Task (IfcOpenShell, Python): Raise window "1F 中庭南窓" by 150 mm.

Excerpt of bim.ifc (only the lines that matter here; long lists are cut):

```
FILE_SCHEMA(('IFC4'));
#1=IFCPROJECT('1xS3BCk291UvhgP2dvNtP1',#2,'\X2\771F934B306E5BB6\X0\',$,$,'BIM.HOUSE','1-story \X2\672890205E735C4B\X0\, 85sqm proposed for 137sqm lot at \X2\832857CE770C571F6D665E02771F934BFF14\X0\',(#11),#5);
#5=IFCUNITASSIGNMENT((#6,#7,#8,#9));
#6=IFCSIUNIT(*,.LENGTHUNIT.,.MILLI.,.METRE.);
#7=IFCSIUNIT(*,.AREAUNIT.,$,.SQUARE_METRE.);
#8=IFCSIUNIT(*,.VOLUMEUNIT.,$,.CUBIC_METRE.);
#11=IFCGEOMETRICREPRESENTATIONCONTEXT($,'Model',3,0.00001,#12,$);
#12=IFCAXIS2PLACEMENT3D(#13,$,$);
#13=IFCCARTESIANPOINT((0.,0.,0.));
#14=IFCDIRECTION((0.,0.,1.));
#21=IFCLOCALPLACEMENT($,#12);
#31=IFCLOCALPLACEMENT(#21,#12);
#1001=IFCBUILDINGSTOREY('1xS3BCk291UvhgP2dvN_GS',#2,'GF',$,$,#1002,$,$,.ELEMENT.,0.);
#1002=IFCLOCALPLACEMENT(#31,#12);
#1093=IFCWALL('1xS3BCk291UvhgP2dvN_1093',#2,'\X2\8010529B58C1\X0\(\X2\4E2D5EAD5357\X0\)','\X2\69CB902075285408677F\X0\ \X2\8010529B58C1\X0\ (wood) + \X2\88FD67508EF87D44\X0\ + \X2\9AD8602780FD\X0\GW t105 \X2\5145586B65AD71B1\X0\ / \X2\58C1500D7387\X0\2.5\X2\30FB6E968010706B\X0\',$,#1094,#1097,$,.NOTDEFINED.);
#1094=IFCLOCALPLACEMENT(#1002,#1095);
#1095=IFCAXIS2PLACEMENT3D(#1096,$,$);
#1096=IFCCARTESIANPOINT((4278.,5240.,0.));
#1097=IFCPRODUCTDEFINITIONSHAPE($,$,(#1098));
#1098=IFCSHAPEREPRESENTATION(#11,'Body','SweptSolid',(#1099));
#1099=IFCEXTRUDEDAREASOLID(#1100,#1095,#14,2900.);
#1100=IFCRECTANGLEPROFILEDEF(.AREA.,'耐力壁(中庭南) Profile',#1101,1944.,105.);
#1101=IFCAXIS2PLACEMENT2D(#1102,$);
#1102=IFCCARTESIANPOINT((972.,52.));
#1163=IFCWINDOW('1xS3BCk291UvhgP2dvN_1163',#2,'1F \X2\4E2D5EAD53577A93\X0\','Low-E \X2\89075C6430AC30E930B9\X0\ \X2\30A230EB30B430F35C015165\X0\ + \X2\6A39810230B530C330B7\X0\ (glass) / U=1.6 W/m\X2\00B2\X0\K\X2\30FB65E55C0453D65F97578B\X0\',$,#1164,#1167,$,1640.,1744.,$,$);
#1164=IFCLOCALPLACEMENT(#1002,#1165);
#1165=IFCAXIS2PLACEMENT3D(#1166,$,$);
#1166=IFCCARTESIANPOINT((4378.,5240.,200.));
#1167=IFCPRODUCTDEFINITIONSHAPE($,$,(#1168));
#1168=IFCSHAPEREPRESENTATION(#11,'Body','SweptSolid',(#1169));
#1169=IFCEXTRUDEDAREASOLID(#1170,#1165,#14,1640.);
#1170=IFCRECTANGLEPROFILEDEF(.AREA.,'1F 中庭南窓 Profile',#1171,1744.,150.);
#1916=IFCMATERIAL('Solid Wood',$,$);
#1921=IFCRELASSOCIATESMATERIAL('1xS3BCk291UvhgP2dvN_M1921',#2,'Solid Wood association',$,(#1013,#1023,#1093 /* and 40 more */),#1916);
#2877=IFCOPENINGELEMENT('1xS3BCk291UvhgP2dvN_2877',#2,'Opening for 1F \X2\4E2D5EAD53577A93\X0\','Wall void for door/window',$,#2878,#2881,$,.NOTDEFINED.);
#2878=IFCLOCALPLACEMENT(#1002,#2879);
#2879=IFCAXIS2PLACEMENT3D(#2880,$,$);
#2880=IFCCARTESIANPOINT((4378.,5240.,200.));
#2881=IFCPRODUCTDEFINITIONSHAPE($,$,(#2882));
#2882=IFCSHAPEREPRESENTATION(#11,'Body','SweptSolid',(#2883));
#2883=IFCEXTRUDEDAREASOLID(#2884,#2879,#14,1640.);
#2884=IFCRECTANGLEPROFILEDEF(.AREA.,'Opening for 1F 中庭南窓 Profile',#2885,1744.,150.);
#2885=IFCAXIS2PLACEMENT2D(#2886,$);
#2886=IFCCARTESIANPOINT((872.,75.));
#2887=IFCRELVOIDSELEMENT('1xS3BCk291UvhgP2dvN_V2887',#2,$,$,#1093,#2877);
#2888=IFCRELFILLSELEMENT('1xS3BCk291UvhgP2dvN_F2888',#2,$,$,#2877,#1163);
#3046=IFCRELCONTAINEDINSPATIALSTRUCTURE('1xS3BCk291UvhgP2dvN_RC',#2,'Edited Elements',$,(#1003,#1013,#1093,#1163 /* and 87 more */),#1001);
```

```python
import numpy as np
import ifcopenshell
import ifcopenshell.api.geometry
import ifcopenshell.util.placement
import ifcopenshell.util.unit

model = ifcopenshell.open("bim.ifc")
unit_scale = ifcopenshell.util.unit.calculate_unit_scale(model)

window = model.by_guid("1xS3BCk291UvhgP2dvN_1163")
opening = window.FillsVoids[0].RelatingOpeningElement
dz = 150.0

shift = np.array([0.0, 0.0, dz])
# The window is not placed relative to its opening, so move both.
for product in (opening, window):
    matrix = ifcopenshell.util.placement.get_local_placement(product.ObjectPlacement)
    matrix[:3, 3] += shift
    ifcopenshell.api.geometry.edit_object_placement(model, product=product, matrix=matrix, is_si=False)

print(f"moved by {dz * unit_scale:+.3f} m")

model.write("bim_edited.ifc")
```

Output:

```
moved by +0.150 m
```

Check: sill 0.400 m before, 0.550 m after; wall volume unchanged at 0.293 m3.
